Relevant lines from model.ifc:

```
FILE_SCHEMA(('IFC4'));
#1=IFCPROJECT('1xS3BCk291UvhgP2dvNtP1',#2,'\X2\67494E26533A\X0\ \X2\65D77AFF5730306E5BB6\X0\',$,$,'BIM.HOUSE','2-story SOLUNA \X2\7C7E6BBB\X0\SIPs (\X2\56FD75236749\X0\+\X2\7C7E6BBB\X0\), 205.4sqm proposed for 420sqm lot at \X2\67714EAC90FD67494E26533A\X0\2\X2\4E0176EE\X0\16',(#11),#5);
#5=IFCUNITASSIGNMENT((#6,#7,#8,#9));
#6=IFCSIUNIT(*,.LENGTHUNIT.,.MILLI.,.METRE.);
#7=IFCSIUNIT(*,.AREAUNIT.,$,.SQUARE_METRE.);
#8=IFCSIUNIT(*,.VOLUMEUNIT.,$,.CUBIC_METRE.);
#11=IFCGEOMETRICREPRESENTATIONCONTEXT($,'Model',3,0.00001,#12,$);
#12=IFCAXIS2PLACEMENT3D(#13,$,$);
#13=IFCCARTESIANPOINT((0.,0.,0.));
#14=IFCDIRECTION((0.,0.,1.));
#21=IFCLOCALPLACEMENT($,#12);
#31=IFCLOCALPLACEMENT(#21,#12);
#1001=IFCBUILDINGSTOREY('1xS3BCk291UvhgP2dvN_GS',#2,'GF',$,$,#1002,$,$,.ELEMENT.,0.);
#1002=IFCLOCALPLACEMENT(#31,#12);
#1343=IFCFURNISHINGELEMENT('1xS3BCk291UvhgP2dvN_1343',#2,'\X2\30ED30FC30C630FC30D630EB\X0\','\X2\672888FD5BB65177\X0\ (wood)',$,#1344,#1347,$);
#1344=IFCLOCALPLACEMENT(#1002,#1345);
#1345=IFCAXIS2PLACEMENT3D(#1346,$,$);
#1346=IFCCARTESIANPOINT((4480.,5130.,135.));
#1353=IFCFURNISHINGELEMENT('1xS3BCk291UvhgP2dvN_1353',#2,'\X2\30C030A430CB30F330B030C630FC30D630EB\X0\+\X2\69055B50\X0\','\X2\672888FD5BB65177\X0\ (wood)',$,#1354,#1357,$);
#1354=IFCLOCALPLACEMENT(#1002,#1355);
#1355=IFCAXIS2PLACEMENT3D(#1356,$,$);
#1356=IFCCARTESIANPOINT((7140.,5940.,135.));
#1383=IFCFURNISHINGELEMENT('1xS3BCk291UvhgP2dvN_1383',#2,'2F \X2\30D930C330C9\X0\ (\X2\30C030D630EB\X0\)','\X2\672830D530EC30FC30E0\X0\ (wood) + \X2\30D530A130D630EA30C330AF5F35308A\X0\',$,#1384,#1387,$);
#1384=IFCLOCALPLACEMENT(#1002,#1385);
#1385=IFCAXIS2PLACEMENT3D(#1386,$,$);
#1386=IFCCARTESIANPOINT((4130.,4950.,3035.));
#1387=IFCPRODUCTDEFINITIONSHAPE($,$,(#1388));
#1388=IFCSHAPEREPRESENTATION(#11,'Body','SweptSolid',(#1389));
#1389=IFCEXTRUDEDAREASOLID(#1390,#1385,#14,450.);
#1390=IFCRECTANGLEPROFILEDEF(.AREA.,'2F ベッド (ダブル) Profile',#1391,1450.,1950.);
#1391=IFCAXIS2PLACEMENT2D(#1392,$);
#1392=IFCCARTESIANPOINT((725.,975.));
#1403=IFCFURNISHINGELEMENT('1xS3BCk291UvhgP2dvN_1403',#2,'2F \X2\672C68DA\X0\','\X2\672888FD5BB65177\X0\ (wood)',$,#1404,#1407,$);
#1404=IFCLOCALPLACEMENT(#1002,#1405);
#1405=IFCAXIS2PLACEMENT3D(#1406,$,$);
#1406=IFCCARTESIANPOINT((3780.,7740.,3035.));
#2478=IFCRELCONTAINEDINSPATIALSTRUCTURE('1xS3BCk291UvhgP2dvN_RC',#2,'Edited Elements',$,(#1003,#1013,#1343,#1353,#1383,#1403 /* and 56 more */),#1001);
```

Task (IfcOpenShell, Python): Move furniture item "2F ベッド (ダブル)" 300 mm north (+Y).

```python
import ifcopenshell
import ifcopenshell.api.geometry
import ifcopenshell.util.placement
import ifcopenshell.util.unit

model = ifcopenshell.open("model.ifc")
unit_scale = ifcopenshell.util.unit.calculate_unit_scale(model)

item = model.by_id(1383)
matrix = ifcopenshell.util.placement.get_local_placement(item.ObjectPlacement)
matrix[1, 3] += 0.3 / unit_scale
ifcopenshell.api.geometry.edit_object_placement(model, product=item, matrix=matrix, is_si=False)

print(ifcopenshell.util.placement.get_local_placement(item.ObjectPlacement).round(3) + 0.0)

model.write("model_updated.ifc")
```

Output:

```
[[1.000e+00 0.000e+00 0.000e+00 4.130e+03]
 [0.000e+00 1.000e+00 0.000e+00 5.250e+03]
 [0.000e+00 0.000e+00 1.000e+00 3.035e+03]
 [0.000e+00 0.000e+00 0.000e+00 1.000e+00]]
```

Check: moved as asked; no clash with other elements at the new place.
